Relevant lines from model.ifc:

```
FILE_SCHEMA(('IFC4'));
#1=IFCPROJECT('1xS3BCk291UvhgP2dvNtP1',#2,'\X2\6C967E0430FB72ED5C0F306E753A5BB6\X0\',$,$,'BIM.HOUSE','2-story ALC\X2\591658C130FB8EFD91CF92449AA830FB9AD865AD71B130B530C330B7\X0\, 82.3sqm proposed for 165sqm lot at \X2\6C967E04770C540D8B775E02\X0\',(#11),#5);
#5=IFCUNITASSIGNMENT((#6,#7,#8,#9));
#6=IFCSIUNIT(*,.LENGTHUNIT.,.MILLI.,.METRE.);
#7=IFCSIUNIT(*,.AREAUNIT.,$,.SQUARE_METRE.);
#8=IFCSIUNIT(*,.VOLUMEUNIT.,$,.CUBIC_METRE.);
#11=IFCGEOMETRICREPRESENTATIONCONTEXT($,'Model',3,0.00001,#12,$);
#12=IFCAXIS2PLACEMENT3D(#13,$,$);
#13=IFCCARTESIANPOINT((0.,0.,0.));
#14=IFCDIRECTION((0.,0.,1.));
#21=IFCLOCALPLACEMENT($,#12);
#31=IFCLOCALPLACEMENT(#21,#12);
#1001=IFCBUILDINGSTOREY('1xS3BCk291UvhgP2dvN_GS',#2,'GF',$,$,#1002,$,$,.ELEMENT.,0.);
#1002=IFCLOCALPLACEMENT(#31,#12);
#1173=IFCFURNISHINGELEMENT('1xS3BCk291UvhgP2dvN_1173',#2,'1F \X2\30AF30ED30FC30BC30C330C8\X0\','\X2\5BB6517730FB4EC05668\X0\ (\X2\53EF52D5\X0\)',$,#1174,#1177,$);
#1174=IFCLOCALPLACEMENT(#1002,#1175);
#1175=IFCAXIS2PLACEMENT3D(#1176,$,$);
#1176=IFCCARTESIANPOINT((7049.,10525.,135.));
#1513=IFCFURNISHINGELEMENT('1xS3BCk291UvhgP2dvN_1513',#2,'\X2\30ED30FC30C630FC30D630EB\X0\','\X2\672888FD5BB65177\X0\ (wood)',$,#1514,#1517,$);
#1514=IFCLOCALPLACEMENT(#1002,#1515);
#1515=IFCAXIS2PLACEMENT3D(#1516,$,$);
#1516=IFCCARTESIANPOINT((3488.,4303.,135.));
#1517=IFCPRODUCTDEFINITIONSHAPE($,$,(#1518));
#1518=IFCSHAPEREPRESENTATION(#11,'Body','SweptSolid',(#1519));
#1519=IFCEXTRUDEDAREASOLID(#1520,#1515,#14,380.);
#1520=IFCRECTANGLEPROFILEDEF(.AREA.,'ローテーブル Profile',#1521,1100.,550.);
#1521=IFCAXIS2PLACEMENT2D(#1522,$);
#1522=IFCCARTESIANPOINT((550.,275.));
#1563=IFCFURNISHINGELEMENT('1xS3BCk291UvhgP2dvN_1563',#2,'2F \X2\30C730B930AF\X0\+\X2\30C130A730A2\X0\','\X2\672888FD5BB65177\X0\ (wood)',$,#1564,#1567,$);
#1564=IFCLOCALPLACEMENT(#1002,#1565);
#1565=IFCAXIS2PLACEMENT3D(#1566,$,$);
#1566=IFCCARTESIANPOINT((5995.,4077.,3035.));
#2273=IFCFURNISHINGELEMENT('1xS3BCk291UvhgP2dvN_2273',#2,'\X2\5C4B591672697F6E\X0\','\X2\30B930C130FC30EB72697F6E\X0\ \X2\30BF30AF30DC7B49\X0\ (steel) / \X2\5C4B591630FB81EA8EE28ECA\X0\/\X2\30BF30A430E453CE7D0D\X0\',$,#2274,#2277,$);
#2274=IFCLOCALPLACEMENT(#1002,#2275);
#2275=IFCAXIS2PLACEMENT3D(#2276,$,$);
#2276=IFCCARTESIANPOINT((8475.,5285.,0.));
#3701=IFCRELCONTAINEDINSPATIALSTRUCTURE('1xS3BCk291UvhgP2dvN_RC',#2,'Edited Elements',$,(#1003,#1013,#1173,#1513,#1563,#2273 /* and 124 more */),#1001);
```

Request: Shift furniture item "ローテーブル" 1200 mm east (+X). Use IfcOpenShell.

```python
import ifcopenshell
import ifcopenshell.api.geometry
import ifcopenshell.util.placement
import ifcopenshell.util.unit

model = ifcopenshell.open("model.ifc")
unit_scale = ifcopenshell.util.unit.calculate_unit_scale(model)

item = model.by_guid("1xS3BCk291UvhgP2dvN_1513")
matrix = ifcopenshell.util.placement.get_local_placement(item.ObjectPlacement)
matrix[0, 3] += 1.2 / unit_scale
ifcopenshell.api.geometry.edit_object_placement(model, product=item, matrix=matrix, is_si=False)

print(ifcopenshell.util.placement.get_local_placement(item.ObjectPlacement).round(3) + 0.0)

model.write("model_edited.ifc")
```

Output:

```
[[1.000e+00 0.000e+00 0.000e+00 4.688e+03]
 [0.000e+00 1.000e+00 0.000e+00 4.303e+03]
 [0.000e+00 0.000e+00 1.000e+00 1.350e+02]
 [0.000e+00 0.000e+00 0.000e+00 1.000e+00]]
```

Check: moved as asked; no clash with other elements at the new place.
